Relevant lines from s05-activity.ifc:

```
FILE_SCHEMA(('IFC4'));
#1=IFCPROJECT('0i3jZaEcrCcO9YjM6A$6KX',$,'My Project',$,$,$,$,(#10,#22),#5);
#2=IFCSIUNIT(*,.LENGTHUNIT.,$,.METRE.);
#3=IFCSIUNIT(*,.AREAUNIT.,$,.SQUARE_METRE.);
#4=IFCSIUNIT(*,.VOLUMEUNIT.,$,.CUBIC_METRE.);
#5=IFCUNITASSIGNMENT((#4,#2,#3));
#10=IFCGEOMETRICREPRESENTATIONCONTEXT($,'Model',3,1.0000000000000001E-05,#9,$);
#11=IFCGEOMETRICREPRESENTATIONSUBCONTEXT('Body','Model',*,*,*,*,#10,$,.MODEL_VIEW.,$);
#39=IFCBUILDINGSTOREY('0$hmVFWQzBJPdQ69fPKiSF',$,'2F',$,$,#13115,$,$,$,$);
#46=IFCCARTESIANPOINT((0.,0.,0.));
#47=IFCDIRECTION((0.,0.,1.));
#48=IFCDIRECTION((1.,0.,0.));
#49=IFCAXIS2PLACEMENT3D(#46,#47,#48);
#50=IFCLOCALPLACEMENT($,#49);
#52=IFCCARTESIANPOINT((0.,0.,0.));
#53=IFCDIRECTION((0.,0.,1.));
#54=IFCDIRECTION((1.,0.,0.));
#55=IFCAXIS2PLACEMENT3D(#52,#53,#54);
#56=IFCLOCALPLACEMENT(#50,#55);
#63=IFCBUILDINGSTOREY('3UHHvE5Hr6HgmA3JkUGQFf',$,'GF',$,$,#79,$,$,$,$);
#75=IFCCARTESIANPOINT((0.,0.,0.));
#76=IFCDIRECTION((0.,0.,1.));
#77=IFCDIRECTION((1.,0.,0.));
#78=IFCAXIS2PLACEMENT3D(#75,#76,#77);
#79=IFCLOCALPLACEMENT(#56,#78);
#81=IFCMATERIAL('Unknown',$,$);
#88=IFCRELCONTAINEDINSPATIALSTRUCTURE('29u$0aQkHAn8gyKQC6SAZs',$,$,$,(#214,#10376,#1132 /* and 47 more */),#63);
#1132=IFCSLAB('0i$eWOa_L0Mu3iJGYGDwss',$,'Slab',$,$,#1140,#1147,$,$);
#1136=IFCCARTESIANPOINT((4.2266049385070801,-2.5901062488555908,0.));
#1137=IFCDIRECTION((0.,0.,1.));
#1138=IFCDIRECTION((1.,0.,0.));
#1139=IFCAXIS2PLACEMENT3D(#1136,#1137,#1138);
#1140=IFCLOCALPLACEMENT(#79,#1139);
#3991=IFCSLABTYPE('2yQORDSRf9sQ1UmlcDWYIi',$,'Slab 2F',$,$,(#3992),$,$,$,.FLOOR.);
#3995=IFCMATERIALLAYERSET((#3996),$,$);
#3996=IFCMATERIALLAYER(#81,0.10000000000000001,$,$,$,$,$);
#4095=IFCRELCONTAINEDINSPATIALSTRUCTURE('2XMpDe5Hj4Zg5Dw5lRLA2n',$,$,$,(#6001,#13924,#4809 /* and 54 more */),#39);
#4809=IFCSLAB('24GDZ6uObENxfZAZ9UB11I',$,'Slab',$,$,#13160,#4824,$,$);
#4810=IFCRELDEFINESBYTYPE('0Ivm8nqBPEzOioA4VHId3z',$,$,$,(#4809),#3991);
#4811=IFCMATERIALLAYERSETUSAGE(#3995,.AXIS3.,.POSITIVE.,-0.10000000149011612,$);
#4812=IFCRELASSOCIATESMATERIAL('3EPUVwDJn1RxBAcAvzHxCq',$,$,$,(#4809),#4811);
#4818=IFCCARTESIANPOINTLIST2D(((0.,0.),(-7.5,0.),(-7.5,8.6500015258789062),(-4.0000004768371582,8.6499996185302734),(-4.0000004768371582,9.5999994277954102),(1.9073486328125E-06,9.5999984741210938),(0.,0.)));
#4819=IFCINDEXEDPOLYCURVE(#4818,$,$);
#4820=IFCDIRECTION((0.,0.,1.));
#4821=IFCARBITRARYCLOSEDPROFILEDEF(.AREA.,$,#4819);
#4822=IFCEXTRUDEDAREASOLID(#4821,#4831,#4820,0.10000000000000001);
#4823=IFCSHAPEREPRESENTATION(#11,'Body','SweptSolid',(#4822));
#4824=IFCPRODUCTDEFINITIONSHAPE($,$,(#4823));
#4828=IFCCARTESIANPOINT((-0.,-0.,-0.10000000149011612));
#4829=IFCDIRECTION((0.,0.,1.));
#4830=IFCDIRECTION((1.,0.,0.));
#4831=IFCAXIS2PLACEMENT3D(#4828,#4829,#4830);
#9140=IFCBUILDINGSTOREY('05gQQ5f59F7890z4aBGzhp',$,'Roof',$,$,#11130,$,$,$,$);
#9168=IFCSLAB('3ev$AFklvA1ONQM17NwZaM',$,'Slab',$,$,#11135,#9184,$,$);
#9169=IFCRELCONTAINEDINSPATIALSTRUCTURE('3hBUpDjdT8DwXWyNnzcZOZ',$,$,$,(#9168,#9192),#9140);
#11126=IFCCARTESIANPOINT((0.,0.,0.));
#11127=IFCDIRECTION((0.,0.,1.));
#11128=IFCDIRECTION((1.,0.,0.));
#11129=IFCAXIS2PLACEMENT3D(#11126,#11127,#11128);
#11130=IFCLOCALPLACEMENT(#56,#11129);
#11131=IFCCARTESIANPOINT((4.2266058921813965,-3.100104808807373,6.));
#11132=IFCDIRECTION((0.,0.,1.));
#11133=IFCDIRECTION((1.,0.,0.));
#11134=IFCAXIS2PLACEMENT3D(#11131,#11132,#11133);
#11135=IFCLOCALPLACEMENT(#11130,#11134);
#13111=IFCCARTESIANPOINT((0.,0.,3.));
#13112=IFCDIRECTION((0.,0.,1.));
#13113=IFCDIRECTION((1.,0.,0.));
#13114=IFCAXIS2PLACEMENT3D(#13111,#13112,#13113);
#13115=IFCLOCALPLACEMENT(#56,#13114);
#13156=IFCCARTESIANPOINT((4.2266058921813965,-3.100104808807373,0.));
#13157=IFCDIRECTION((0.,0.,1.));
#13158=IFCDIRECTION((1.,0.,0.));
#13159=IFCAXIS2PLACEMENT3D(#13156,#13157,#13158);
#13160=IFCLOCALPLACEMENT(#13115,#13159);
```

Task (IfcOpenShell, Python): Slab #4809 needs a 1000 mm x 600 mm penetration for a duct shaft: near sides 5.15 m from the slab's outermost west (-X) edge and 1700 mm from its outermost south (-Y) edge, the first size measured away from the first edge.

```python
import numpy as np
import ifcopenshell
import ifcopenshell.api.feature
import ifcopenshell.api.geometry
import ifcopenshell.api.root
import ifcopenshell.geom
import ifcopenshell.util.placement
import ifcopenshell.util.representation
import ifcopenshell.util.shape
import ifcopenshell.util.unit

model = ifcopenshell.open("s05-activity.ifc")
unit_scale = ifcopenshell.util.unit.calculate_unit_scale(model)
settings = ifcopenshell.geom.settings()


def volume(element):
    """Net volume in cubic metres, openings subtracted."""
    shape = ifcopenshell.geom.create_shape(settings, element)
    return ifcopenshell.util.shape.get_volume(shape.geometry)


slab = model.by_id(4809)
before = volume(slab)

# Extent in the slab's own axes, in metres. The edges named are its -X and -Y sides.
slab_shape = ifcopenshell.geom.create_shape(settings, slab)
vertices = ifcopenshell.util.shape.get_vertices(slab_shape.geometry)
x_min, y_min, bottom = vertices.min(axis=0)
top = vertices[:, 2].max()

opening = ifcopenshell.api.root.create_entity(model, ifc_class="IfcOpeningElement", name="Duct shaft opening", predefined_type="OPENING")
context = ifcopenshell.util.representation.get_context(model, "Model", "Body", "MODEL_VIEW")
width, depth = 1, 0.6
outline = [(0.0, 0.0), (width, 0.0), (width, depth), (0.0, depth), (0.0, 0.0)]
# Overshoot both faces by 50 mm so the cut is clean.
shape = ifcopenshell.api.geometry.add_slab_representation(
    model, context=context, depth=top - bottom + 0.1, polyline=outline
)
ifcopenshell.api.geometry.assign_representation(model, product=opening, representation=shape)

matrix = ifcopenshell.util.placement.get_local_placement(slab.ObjectPlacement)
matrix[:, 3] = matrix @ np.append(np.array([x_min + 5.15, y_min + 1.7, bottom - 0.05]) / unit_scale, 1.0)
ifcopenshell.api.geometry.edit_object_placement(model, product=opening, matrix=matrix, is_si=False)
ifcopenshell.api.feature.add_feature(model, feature=opening, element=slab)

after = volume(slab)

print(f"slab volume {before:.3f} -> {after:.3f} m3")

model.write("s05-activity-out.ifc")
```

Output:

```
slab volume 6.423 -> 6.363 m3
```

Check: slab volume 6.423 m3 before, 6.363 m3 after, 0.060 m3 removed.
